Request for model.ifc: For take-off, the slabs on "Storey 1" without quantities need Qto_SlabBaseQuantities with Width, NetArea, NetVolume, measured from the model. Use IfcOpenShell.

First a look at what the model holds.

```python
import ifcopenshell
import ifcopenshell.util.element
import ifcopenshell.util.unit

model = ifcopenshell.open("model.ifc")
print(model.schema)
for unit_type in ("LENGTHUNIT", "AREAUNIT", "VOLUMEUNIT"):
    print(unit_type, ifcopenshell.util.unit.calculate_unit_scale(model, unit_type))
storey = next(s for s in model.by_type("IfcBuildingStorey") if s.Name == "Storey 1")
slabs = [e for e in ifcopenshell.util.element.get_decomposition(storey) if e.is_a("IfcSlab")]
for e in sorted(slabs, key=lambda e: e.id()):
    print(e.id(), e.is_a(), e.Name, list(ifcopenshell.util.element.get_psets(e, qtos_only=True)), sep=" | ")
```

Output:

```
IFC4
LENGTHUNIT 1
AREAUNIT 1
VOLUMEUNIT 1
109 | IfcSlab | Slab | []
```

```python
import ifcopenshell
import ifcopenshell.api.pset
import ifcopenshell.geom
import ifcopenshell.util.element
import ifcopenshell.util.shape
import ifcopenshell.util.unit

model = ifcopenshell.open("model.ifc")
unit_scale = ifcopenshell.util.unit.calculate_unit_scale(model)
area_scale = ifcopenshell.util.unit.calculate_unit_scale(model, "AREAUNIT")
volume_scale = ifcopenshell.util.unit.calculate_unit_scale(model, "VOLUMEUNIT")
settings = ifcopenshell.geom.settings()

storey = next(s for s in model.by_type("IfcBuildingStorey") if s.Name == "Storey 1")
slabs = [e for e in ifcopenshell.util.element.get_decomposition(storey) if e.is_a("IfcSlab")]

for e in sorted(slabs, key=lambda e: e.id()):
    if ifcopenshell.util.element.get_psets(e, qtos_only=True, should_inherit=False):
        continue
    # Geometry comes back in metres, in the element's own axes.
    shape = ifcopenshell.geom.create_shape(settings, e)
    values = {
        "Width": ifcopenshell.util.shape.get_z(shape.geometry) / unit_scale,
        "NetArea": ifcopenshell.util.shape.get_footprint_area(shape.geometry) / area_scale,
        "NetVolume": ifcopenshell.util.shape.get_volume(shape.geometry) / volume_scale,
    }
    qto = ifcopenshell.api.pset.add_qto(model, product=e, name="Qto_SlabBaseQuantities")
    ifcopenshell.api.pset.edit_qto(model, qto=qto, properties=values)
    print(e.id(), {k: round(v, 3) for k, v in values.items()})

model.write("model-out.ifc")
```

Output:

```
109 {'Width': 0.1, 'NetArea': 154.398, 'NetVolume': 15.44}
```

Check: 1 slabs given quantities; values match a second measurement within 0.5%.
